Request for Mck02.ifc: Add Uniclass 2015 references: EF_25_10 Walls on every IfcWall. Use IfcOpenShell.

First a look at what the model holds.

```python
import ifcopenshell

model = ifcopenshell.open("Mck02.ifc")
print(model.schema)
print("classifications:", [c.Name for c in model.by_type("IfcClassification")])
for ifc_class in ("IfcDoor", "IfcRoof", "IfcStair", "IfcWall", "IfcWindow"):
    print(ifc_class, len(model.by_type(ifc_class)))
```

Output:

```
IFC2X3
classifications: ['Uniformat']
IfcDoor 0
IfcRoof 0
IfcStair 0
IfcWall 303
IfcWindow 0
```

```python
import ifcopenshell
import ifcopenshell.api.classification

model = ifcopenshell.open("Mck02.ifc")

# IFC2X3 requires Source and Edition and has no link from the project to the system.
system = model.create_entity("IfcClassification", Source="NBS", Edition="2015", Name="Uniclass 2015")

codes = {
    "IfcWall": ("EF_25_10", "Walls"),
}
for ifc_class, (code, name) in codes.items():
    products = model.by_type(ifc_class)
    ifcopenshell.api.classification.add_reference(
        model, products=products, classification=system, identification=code, name=name
    )
    print(code, len(products))

model.write("Mck02_edited.ifc")
```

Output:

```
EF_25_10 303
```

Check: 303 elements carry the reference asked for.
